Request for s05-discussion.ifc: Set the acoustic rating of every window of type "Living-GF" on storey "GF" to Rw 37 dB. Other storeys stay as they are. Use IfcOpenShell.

First a look at what the model holds.

```python
import ifcopenshell
import ifcopenshell.util.element

model = ifcopenshell.open("s05-discussion.ifc")
print(model.schema)
storey = next(s for s in model.by_type("IfcBuildingStorey") if s.Name == "GF")
windows = [e for e in ifcopenshell.util.element.get_decomposition(storey) if e.is_a("IfcWindow")]
seen = {}
for e in windows:
    element_type = ifcopenshell.util.element.get_type(e)
    key = (element_type.Name if element_type != e and element_type else None, ifcopenshell.util.element.get_pset(e, "Pset_WindowCommon", "AcousticRating"))
    seen[key] = seen.get(key, 0) + 1
for (name, value), count in sorted(seen.items(), key=str):
    print(count, "x", name, "|", value)
```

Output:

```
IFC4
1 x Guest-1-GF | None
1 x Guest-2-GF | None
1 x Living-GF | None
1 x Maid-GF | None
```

```python
import ifcopenshell
import ifcopenshell.api.pset
import ifcopenshell.util.element

model = ifcopenshell.open("s05-discussion.ifc")

storey = next(s for s in model.by_type("IfcBuildingStorey") if s.Name == "GF")
windows = [e for e in ifcopenshell.util.element.get_decomposition(storey) if e.is_a("IfcWindow")]

count = 0
for e in windows:
    element_type = ifcopenshell.util.element.get_type(e)
    if element_type in (None, e) or element_type.Name != "Living-GF":
        continue
    # add_pset returns the element's existing set when there is one.
    pset = ifcopenshell.api.pset.add_pset(model, product=e, name="Pset_WindowCommon")
    ifcopenshell.api.pset.edit_pset(model, pset=pset, properties={"AcousticRating": "Rw 37 dB"})
    count += 1

print(count, "windows updated")

model.write("s05-discussion-out.ifc")
```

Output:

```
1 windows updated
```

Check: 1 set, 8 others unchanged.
